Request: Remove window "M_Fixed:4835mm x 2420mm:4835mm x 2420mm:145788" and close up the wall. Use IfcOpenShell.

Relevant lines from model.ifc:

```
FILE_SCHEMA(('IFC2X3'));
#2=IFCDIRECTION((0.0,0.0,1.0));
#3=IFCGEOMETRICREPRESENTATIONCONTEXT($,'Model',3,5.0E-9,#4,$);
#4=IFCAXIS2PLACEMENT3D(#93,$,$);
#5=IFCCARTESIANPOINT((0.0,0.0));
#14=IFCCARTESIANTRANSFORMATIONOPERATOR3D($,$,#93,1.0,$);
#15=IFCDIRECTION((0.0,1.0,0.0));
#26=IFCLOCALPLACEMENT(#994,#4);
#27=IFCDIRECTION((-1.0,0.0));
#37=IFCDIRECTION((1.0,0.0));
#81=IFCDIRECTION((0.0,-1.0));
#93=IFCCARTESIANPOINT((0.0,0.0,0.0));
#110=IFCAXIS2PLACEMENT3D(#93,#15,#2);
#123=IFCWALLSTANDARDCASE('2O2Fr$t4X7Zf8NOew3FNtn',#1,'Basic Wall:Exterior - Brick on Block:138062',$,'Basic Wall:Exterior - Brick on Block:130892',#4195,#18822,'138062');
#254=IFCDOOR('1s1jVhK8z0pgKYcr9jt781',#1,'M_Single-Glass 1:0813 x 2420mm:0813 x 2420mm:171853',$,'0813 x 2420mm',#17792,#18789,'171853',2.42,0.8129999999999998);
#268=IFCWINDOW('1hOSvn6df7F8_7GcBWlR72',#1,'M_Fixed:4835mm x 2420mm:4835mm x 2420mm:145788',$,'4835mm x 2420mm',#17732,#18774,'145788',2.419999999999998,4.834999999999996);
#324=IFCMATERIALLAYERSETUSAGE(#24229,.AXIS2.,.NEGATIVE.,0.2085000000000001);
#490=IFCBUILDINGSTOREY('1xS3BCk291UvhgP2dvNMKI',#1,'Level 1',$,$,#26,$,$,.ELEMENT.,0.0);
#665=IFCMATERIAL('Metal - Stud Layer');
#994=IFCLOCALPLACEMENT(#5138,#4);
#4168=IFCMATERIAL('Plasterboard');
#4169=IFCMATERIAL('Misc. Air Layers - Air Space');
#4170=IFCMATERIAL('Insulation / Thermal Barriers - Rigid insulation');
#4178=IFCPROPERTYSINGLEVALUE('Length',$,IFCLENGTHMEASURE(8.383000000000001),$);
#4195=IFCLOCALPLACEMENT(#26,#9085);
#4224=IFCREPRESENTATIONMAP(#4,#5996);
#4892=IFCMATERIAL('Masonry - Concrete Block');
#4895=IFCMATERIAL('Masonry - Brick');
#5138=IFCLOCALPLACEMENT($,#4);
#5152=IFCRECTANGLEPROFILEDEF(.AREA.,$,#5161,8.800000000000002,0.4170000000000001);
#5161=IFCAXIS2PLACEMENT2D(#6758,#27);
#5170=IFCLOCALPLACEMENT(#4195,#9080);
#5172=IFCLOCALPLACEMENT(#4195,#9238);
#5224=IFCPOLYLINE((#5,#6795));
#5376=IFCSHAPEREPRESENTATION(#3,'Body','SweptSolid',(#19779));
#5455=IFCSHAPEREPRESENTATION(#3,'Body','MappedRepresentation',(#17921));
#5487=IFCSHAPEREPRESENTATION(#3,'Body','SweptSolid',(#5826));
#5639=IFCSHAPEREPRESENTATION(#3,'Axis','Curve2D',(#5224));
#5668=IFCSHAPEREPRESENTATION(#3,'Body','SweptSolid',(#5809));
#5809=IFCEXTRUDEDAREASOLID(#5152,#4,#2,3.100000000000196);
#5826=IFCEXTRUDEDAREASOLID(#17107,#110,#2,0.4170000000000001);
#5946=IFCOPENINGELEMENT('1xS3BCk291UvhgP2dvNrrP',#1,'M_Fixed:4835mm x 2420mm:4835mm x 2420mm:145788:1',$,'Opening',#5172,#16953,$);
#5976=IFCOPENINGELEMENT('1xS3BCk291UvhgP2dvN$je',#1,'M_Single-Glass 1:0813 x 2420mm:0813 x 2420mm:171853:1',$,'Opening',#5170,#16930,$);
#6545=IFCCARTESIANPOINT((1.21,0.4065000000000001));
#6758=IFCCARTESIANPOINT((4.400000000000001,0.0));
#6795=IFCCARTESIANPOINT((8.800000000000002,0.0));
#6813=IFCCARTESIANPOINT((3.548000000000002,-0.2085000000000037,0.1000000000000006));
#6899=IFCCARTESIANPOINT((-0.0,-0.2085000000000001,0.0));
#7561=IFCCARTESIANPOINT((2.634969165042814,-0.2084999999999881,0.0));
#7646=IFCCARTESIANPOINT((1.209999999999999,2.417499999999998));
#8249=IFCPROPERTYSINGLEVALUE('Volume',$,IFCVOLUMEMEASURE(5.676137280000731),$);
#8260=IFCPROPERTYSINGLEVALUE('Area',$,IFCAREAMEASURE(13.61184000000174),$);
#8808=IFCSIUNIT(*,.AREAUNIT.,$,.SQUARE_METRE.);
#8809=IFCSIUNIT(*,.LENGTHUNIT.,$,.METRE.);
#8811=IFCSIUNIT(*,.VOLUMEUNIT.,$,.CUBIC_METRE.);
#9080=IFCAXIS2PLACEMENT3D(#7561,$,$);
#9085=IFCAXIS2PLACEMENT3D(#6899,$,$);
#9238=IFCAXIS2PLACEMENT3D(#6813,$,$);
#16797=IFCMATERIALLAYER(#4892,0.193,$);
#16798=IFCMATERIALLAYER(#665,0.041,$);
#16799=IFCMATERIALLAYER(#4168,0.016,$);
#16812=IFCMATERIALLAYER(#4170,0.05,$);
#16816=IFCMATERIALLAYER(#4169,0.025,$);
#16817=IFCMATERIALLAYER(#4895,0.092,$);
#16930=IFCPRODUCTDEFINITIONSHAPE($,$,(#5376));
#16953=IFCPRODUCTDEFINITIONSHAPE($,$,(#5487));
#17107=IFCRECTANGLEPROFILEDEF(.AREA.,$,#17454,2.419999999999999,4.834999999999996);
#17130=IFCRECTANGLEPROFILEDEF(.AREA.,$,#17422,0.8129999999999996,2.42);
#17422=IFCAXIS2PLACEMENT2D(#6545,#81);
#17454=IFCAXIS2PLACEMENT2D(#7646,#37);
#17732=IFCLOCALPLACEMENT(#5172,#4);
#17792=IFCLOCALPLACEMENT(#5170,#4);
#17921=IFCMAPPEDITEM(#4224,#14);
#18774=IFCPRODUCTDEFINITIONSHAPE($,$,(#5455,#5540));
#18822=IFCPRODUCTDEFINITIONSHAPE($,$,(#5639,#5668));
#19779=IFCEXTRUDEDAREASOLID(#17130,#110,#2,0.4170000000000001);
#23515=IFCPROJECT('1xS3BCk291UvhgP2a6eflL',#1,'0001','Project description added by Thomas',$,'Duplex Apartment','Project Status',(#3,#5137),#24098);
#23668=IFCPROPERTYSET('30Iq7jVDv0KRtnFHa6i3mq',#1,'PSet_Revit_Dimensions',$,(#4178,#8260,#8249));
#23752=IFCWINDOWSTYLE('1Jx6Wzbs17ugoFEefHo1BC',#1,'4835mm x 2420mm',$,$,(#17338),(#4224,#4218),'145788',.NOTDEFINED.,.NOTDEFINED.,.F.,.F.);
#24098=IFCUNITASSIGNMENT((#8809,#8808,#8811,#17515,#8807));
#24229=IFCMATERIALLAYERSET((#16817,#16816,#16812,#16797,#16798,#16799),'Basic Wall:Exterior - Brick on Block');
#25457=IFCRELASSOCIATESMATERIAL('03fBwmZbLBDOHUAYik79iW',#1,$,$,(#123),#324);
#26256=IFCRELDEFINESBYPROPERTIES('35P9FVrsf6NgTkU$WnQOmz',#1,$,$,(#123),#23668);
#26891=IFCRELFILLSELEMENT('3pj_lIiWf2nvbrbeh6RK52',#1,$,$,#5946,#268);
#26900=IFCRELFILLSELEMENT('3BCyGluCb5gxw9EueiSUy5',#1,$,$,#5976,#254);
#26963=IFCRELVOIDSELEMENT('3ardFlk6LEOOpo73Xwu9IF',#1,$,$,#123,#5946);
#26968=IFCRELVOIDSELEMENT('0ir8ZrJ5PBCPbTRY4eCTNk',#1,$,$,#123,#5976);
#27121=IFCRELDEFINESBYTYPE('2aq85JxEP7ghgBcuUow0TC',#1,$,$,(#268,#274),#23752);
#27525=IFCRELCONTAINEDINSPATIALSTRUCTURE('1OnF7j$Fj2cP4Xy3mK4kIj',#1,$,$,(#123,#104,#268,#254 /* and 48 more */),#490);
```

```python
import ifcopenshell
import ifcopenshell.api.feature
import ifcopenshell.api.pset
import ifcopenshell.api.root
import ifcopenshell.geom
import ifcopenshell.util.element
import ifcopenshell.util.shape
import ifcopenshell.util.unit

model = ifcopenshell.open("model.ifc")
area_scale = ifcopenshell.util.unit.calculate_unit_scale(model, "AREAUNIT")
volume_scale = ifcopenshell.util.unit.calculate_unit_scale(model, "VOLUMEUNIT")
settings = ifcopenshell.geom.settings()


def volume(element):
    """Net volume in cubic metres, openings subtracted."""
    shape = ifcopenshell.geom.create_shape(settings, element)
    return ifcopenshell.util.shape.get_volume(shape.geometry)


window = model.by_guid("1hOSvn6df7F8_7GcBWlR72")
opening = window.FillsVoids[0].RelatingOpeningElement
wall = opening.VoidsElements[0].RelatingBuildingElement
before = volume(wall)

ifcopenshell.api.root.remove_product(model, product=window)
ifcopenshell.api.feature.remove_feature(model, feature=opening)

after = volume(wall)
thickness = 0.417  # wall thickness in metres

# Update the wall's stored quantities.
pset = model.by_id(ifcopenshell.util.element.get_pset(wall, "PSet_Revit_Dimensions", should_inherit=False)["id"])
ifcopenshell.api.pset.edit_pset(model, pset=pset, properties={
    "Area": model.create_entity("IfcAreaMeasure", after / thickness / area_scale),
    "Volume": model.create_entity("IfcVolumeMeasure", after / volume_scale),
})

print(f"wall volume {before:.3f} -> {after:.3f} m3")

model.write("model_v2.ifc")
```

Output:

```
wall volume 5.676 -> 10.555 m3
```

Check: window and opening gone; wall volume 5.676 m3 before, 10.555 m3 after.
